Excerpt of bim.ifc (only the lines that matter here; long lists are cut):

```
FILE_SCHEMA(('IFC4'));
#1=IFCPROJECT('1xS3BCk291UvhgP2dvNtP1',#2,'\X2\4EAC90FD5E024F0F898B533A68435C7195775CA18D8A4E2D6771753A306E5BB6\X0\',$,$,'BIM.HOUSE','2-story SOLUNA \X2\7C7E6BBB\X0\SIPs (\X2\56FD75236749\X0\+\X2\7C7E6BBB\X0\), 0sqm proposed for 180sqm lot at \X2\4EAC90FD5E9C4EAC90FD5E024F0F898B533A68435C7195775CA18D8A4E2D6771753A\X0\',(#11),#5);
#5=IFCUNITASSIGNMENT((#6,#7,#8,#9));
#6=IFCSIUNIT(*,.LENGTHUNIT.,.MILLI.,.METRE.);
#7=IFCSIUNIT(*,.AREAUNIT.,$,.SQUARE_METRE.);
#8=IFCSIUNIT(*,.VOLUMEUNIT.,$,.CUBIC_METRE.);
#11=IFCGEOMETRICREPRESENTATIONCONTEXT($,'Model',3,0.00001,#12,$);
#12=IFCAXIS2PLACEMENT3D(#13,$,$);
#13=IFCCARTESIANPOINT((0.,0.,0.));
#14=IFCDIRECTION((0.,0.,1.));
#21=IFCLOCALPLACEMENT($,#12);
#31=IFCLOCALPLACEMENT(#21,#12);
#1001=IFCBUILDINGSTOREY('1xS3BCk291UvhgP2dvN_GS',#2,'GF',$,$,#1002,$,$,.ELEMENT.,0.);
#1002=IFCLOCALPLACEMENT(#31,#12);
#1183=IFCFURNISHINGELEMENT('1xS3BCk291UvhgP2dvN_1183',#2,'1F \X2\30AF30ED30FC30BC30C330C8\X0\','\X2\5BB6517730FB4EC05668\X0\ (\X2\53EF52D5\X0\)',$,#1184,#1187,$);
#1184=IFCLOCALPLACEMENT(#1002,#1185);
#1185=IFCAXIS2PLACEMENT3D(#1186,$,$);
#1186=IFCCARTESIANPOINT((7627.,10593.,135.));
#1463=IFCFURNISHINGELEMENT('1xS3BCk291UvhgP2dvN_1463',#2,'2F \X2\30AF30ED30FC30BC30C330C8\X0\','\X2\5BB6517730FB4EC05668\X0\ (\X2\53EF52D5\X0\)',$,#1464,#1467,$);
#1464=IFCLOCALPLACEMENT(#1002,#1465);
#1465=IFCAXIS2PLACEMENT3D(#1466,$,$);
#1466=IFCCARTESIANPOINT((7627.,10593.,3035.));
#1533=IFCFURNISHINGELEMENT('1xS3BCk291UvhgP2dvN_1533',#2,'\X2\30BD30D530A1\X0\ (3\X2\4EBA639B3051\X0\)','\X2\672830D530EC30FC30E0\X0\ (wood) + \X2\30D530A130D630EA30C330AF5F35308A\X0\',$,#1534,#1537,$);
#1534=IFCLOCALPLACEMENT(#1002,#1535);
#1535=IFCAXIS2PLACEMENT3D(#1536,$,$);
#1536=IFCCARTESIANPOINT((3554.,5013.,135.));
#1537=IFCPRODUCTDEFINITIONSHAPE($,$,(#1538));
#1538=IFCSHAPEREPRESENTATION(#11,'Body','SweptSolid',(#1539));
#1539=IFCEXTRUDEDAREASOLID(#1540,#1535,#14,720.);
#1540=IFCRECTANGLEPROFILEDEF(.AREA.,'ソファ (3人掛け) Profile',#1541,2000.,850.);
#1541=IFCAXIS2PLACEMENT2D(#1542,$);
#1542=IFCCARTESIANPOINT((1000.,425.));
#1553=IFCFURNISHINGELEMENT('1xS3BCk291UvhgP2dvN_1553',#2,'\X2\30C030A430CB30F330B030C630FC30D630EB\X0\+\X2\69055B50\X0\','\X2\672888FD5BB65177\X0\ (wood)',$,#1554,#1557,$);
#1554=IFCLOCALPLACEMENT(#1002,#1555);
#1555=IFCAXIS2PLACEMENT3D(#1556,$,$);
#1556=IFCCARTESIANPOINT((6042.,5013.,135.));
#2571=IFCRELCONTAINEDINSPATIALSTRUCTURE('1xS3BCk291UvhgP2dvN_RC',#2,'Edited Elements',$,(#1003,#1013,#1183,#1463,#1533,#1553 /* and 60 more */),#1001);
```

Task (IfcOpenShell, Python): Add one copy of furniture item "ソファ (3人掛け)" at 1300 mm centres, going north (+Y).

```python
import numpy as np
import ifcopenshell
import ifcopenshell.api.geometry
import ifcopenshell.api.root
import ifcopenshell.util.element
import ifcopenshell.util.placement

model = ifcopenshell.open("bim.ifc")


def reuse_history(source, copy):
    """copy_class also copies each property set's owner history, people and application; keep the originals."""
    for rel in copy.IsDefinedBy:
        if rel.is_a("IfcRelDefinesByProperties") and (history := rel.RelatingPropertyDefinition.OwnerHistory):
            rel.RelatingPropertyDefinition.OwnerHistory = source.OwnerHistory
            ifcopenshell.util.element.remove_deep2(model, history)


source = model.by_guid("1xS3BCk291UvhgP2dvN_1533")
base = ifcopenshell.util.placement.get_local_placement(source.ObjectPlacement)
step = np.array([0.0, 1.0, 0.0]) * 1300.0

for i in range(1, 2):
    copy = ifcopenshell.api.root.copy_class(model, product=source)
    copy.Representation = ifcopenshell.util.element.copy_deep(
        model, source.Representation, exclude=["IfcGeometricRepresentationContext", "IfcRepresentationMap"]
    )
    reuse_history(source, copy)
    matrix = base.copy()
    matrix[:3, 3] += i * step
    print("added at", matrix[:3, 3].round(3) + 0.0)
    ifcopenshell.api.geometry.edit_object_placement(model, product=copy, matrix=matrix, is_si=False)

model.write("bim_rev.ifc")
```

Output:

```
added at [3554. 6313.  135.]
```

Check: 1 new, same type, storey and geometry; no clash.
